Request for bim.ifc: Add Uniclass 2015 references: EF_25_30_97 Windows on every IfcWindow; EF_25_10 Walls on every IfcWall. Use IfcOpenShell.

First a look at what the model holds.

```python
import ifcopenshell

model = ifcopenshell.open("bim.ifc")
print(model.schema)
print("classifications:", [c.Name for c in model.by_type("IfcClassification")])
for ifc_class in ("IfcDoor", "IfcRoof", "IfcStair", "IfcWall", "IfcWindow"):
    print(ifc_class, len(model.by_type(ifc_class)))
```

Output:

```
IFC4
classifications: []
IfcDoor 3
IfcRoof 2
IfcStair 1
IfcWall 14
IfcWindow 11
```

```python
import ifcopenshell
import ifcopenshell.api.classification

model = ifcopenshell.open("bim.ifc")

system = ifcopenshell.api.classification.add_classification(model, classification="Uniclass 2015")

codes = {
    "IfcWindow": ("EF_25_30_97", "Windows"),
    "IfcWall": ("EF_25_10", "Walls"),
}
for ifc_class, (code, name) in codes.items():
    products = model.by_type(ifc_class)
    ifcopenshell.api.classification.add_reference(
        model, products=products, classification=system, identification=code, name=name
    )
    print(code, len(products))

model.write("bim-out.ifc")
```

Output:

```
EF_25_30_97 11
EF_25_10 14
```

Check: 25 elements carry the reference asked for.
